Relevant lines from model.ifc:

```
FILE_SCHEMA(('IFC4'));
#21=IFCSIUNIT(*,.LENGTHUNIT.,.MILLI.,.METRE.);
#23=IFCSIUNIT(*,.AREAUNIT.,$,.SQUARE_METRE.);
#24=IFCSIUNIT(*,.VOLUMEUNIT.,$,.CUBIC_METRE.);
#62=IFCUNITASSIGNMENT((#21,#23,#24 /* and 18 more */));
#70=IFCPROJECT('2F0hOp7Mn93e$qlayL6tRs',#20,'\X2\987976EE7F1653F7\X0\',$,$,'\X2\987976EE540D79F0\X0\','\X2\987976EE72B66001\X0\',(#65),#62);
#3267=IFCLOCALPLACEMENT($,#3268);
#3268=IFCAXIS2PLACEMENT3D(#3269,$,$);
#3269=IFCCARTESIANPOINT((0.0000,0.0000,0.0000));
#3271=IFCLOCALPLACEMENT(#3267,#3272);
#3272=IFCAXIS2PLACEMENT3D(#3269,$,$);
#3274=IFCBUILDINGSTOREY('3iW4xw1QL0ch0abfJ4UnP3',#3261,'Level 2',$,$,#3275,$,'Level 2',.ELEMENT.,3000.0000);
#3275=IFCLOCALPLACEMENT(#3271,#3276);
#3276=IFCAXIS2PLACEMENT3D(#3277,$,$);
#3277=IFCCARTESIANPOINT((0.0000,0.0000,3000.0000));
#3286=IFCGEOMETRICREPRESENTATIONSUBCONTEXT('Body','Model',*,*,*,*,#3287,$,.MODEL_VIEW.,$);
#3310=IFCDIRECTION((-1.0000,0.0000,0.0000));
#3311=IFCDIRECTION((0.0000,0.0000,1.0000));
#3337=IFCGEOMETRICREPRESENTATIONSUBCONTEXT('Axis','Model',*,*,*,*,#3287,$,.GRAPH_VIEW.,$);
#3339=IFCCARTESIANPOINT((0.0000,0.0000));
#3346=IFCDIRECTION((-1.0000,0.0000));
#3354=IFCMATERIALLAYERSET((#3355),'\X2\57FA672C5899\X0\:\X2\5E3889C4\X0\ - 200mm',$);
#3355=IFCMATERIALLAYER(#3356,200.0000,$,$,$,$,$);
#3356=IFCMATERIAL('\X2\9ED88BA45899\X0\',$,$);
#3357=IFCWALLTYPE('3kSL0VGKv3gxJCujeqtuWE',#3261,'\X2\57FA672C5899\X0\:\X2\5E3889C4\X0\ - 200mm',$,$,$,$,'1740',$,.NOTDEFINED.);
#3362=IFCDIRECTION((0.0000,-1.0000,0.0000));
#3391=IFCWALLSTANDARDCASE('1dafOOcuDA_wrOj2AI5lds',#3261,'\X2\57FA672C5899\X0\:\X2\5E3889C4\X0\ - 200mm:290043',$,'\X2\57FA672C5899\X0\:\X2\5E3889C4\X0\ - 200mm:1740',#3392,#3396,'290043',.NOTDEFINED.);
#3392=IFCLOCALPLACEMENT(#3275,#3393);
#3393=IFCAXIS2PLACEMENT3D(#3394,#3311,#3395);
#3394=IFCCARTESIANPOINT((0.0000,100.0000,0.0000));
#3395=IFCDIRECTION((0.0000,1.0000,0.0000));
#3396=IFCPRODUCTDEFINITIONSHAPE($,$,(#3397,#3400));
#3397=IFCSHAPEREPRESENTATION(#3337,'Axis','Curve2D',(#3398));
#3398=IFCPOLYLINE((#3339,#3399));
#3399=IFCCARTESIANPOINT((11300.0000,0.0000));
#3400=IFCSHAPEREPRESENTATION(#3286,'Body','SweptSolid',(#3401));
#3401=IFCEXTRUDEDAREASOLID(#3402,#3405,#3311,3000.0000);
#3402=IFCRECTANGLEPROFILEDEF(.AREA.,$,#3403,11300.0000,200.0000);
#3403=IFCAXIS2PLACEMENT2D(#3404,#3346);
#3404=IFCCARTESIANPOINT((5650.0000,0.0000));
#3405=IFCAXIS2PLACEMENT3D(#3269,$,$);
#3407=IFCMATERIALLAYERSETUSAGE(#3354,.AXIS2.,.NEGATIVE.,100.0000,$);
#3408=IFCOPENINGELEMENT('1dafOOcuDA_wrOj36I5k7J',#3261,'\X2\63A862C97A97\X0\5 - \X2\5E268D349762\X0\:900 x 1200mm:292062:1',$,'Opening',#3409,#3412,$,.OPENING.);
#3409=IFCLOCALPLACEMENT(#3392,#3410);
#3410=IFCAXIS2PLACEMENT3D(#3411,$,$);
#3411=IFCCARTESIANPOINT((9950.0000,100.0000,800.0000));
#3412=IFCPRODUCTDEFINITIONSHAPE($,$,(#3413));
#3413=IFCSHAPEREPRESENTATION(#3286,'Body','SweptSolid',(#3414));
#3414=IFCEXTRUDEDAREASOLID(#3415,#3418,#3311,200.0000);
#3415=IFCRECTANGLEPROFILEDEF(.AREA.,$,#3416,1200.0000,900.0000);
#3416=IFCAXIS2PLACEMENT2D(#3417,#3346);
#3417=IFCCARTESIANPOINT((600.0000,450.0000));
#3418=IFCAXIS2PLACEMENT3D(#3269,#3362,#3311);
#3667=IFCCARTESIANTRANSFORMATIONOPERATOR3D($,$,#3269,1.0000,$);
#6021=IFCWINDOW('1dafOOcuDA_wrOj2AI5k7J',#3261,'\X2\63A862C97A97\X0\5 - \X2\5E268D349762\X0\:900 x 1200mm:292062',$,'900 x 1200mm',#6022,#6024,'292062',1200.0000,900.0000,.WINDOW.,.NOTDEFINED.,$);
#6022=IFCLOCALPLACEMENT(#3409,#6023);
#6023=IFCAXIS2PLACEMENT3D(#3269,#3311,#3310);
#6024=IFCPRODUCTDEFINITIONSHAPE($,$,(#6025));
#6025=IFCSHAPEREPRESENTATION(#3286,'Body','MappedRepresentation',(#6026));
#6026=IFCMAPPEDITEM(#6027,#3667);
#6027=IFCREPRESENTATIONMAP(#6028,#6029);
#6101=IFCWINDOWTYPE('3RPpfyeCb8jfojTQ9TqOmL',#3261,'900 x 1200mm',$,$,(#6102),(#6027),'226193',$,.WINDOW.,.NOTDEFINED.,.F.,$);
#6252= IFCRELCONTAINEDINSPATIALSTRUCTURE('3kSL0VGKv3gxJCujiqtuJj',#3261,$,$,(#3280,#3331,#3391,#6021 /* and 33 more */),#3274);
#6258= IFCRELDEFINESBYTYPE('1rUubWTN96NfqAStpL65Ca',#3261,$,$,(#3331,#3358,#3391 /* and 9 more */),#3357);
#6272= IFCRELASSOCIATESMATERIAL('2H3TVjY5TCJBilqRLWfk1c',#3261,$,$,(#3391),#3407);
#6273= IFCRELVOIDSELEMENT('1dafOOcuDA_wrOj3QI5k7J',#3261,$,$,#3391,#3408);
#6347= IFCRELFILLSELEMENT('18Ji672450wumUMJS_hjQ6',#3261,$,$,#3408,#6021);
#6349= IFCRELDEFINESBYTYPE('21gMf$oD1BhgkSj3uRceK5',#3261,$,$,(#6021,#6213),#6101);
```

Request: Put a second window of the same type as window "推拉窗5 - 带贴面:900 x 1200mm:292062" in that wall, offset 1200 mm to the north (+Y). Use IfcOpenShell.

```python
import ifcopenshell
import ifcopenshell.api.feature
import ifcopenshell.api.geometry
import ifcopenshell.api.root
import ifcopenshell.geom
import ifcopenshell.util.element
import ifcopenshell.util.placement
import ifcopenshell.util.shape
import ifcopenshell.util.unit

model = ifcopenshell.open("model.ifc")
unit_scale = ifcopenshell.util.unit.calculate_unit_scale(model)
settings = ifcopenshell.geom.settings()


def volume(element):
    """Net volume in cubic metres, openings subtracted."""
    shape = ifcopenshell.geom.create_shape(settings, element)
    return ifcopenshell.util.shape.get_volume(shape.geometry)


def reuse_history(source, copy):
    """copy_class also copies each property set's owner history, people and application; keep the originals."""
    for rel in copy.IsDefinedBy:
        if rel.is_a("IfcRelDefinesByProperties") and (history := rel.RelatingPropertyDefinition.OwnerHistory):
            rel.RelatingPropertyDefinition.OwnerHistory = source.OwnerHistory
            ifcopenshell.util.element.remove_deep2(model, history)


window = model.by_id(6021)
opening = window.FillsVoids[0].RelatingOpeningElement
wall = opening.VoidsElements[0].RelatingBuildingElement
before = volume(wall)
shift = ifcopenshell.util.placement.get_local_placement(wall.ObjectPlacement)[:3, 0] * 1.2 / unit_scale

# copy_class copies the void relationship, type, container and properties, but no geometry.
new_opening = ifcopenshell.api.root.copy_class(model, product=opening)
new_opening.Representation = ifcopenshell.util.element.copy_deep(
    model, opening.Representation, exclude=["IfcGeometricRepresentationContext", "IfcRepresentationMap"]
)
new_opening.Name = "推拉窗5 - 带贴面:900 x 1200mm"
new_window = ifcopenshell.api.root.copy_class(model, product=window)
new_window.Representation = ifcopenshell.util.element.copy_deep(
    model, window.Representation, exclude=["IfcGeometricRepresentationContext", "IfcRepresentationMap"]
)
new_window.Name = "推拉窗5 - 带贴面:900 x 1200mm"
new_window.Tag = None
reuse_history(window, new_window)
ifcopenshell.api.feature.add_filling(model, opening=new_opening, element=new_window)

for old, new in ((opening, new_opening), (window, new_window)):
    matrix = ifcopenshell.util.placement.get_local_placement(old.ObjectPlacement)
    matrix[:3, 3] += shift
    ifcopenshell.api.geometry.edit_object_placement(model, product=new, matrix=matrix, is_si=False)

after = volume(wall)

print(f"wall volume {before:.3f} -> {after:.3f} m3")

model.write("model-out.ifc")
```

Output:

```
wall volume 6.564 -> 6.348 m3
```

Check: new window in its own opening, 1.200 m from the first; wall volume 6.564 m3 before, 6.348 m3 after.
